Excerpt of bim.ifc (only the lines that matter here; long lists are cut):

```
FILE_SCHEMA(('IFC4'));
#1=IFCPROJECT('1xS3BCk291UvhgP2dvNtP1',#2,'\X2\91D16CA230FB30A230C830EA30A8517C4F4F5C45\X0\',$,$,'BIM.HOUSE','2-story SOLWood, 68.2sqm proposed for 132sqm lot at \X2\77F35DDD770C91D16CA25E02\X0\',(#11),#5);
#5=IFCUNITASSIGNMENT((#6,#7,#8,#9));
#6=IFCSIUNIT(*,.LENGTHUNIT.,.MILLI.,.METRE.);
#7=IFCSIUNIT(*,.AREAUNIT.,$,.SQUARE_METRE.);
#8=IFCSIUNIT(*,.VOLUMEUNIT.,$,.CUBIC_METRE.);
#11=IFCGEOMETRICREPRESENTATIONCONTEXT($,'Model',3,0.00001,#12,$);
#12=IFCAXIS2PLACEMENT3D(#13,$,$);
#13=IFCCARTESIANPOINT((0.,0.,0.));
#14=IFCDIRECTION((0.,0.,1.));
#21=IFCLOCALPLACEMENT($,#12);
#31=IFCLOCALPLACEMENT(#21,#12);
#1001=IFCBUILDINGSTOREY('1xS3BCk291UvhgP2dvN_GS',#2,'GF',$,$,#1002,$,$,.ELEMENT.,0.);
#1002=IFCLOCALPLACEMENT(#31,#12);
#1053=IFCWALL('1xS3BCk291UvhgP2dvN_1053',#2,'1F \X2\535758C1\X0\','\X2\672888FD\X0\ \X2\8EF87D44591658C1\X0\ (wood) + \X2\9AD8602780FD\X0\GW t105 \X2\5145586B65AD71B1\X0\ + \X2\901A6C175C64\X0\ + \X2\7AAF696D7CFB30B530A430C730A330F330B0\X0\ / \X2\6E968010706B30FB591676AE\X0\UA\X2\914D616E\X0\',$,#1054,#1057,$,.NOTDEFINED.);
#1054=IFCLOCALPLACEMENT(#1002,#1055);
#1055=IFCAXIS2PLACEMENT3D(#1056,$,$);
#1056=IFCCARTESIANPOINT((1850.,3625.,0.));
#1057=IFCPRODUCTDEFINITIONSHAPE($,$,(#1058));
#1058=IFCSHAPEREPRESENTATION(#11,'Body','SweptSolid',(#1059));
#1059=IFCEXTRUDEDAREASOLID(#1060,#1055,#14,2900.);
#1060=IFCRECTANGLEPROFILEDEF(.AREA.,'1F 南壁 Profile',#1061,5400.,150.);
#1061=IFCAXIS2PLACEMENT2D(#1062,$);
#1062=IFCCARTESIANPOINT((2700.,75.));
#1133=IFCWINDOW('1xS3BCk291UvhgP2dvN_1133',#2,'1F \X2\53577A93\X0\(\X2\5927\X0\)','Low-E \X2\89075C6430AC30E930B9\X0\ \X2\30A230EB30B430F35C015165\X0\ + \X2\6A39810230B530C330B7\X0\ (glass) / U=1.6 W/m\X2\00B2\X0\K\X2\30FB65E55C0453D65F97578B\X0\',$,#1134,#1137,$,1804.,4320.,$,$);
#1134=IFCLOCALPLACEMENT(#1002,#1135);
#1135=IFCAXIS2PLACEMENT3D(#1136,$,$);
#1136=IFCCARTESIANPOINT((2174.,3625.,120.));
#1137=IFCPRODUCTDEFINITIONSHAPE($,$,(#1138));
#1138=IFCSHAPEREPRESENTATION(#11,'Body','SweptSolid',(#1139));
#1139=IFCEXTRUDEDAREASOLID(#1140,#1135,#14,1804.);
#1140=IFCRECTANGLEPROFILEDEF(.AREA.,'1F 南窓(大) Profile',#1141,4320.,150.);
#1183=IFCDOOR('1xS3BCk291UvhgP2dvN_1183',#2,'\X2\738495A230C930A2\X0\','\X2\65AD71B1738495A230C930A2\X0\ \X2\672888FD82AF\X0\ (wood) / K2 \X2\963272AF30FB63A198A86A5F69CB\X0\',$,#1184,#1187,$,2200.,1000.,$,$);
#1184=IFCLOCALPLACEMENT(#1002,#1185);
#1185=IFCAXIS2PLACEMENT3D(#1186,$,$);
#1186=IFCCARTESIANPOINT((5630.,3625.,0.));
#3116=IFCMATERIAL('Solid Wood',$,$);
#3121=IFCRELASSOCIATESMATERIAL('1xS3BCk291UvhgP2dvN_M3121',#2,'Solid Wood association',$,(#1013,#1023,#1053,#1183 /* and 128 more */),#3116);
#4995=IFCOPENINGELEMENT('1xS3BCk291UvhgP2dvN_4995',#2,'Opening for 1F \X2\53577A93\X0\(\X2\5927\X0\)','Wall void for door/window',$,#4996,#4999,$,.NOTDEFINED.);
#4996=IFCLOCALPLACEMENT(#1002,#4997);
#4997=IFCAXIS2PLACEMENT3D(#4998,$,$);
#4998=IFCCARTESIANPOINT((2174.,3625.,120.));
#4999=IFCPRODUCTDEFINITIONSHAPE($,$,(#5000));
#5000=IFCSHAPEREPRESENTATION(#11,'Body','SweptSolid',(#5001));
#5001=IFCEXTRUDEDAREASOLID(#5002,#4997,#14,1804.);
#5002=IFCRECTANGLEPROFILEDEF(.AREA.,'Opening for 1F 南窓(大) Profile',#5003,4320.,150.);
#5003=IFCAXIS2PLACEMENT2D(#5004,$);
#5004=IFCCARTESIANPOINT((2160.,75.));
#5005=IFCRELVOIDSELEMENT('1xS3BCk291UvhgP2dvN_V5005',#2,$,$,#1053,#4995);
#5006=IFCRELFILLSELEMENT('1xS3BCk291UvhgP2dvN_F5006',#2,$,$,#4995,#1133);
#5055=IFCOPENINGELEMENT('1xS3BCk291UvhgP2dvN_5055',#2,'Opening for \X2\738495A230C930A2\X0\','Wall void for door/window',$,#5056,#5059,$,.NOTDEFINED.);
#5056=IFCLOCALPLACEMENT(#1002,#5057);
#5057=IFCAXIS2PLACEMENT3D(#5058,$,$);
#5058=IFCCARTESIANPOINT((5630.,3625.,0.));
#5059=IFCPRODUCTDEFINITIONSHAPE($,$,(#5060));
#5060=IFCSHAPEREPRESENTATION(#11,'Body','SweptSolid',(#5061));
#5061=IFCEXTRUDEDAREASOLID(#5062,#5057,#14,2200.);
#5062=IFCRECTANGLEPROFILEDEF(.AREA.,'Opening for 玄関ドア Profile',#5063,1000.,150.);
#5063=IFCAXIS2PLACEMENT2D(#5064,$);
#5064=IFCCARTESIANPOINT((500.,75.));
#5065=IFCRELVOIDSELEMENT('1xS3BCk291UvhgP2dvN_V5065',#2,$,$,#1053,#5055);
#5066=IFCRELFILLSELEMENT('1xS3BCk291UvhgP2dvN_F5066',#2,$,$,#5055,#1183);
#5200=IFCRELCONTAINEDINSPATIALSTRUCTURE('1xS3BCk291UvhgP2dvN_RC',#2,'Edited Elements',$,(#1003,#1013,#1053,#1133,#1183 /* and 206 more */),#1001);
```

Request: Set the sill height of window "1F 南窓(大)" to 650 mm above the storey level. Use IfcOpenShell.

```python
import numpy as np
import ifcopenshell
import ifcopenshell.api.geometry
import ifcopenshell.geom
import ifcopenshell.util.element
import ifcopenshell.util.placement
import ifcopenshell.util.shape
import ifcopenshell.util.unit

model = ifcopenshell.open("bim.ifc")
unit_scale = ifcopenshell.util.unit.calculate_unit_scale(model)

window = model.by_guid("1xS3BCk291UvhgP2dvN_1133")
opening = window.FillsVoids[0].RelatingOpeningElement
storey = ifcopenshell.util.element.get_container(window, ifc_class="IfcBuildingStorey")
level = ifcopenshell.util.placement.get_local_placement(storey.ObjectPlacement)[2, 3]

# The opening's origin need not be at the sill, so measure its lowest point.
shape = ifcopenshell.geom.create_shape(ifcopenshell.geom.settings(), opening)
bottom = ifcopenshell.util.shape.get_shape_bottom_elevation(shape, shape.geometry) / unit_scale
dz = level + 0.65 / unit_scale - bottom

shift = np.array([0.0, 0.0, dz])
# The window is not placed relative to its opening, so move both.
for product in (opening, window):
    matrix = ifcopenshell.util.placement.get_local_placement(product.ObjectPlacement)
    matrix[:3, 3] += shift
    ifcopenshell.api.geometry.edit_object_placement(model, product=product, matrix=matrix, is_si=False)

print(f"moved by {dz * unit_scale:+.3f} m")

model.write("bim_v2.ifc")
```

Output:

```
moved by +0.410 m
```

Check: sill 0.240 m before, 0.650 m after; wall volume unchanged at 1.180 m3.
